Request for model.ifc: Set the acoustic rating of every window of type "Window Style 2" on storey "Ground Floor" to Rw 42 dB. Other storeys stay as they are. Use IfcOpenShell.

First a look at what the model holds.

```python
import ifcopenshell
import ifcopenshell.util.element

model = ifcopenshell.open("model.ifc")
print(model.schema)
storey = next(s for s in model.by_type("IfcBuildingStorey") if s.Name == "Ground Floor")
windows = [e for e in ifcopenshell.util.element.get_decomposition(storey) if e.is_a("IfcWindow")]
seen = {}
for e in windows:
    element_type = ifcopenshell.util.element.get_type(e)
    key = (element_type.Name if element_type != e and element_type else None, ifcopenshell.util.element.get_pset(e, "Pset_WindowCommon", "AcousticRating"))
    seen[key] = seen.get(key, 0) + 1
for (name, value), count in sorted(seen.items(), key=str):
    print(count, "x", name, "|", value)
```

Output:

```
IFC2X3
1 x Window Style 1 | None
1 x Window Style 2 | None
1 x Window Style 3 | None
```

```python
import ifcopenshell
import ifcopenshell.api.pset
import ifcopenshell.util.element

model = ifcopenshell.open("model.ifc")

storey = next(s for s in model.by_type("IfcBuildingStorey") if s.Name == "Ground Floor")
windows = [e for e in ifcopenshell.util.element.get_decomposition(storey) if e.is_a("IfcWindow")]

count = 0
for e in windows:
    element_type = ifcopenshell.util.element.get_type(e)
    if element_type in (None, e) or element_type.Name != "Window Style 2":
        continue
    # add_pset returns the element's existing set when there is one.
    pset = ifcopenshell.api.pset.add_pset(model, product=e, name="Pset_WindowCommon")
    ifcopenshell.api.pset.edit_pset(model, pset=pset, properties={"AcousticRating": "Rw 42 dB"})
    count += 1

print(count, "windows updated")

model.write("model_v2.ifc")
```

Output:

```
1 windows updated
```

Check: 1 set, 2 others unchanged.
